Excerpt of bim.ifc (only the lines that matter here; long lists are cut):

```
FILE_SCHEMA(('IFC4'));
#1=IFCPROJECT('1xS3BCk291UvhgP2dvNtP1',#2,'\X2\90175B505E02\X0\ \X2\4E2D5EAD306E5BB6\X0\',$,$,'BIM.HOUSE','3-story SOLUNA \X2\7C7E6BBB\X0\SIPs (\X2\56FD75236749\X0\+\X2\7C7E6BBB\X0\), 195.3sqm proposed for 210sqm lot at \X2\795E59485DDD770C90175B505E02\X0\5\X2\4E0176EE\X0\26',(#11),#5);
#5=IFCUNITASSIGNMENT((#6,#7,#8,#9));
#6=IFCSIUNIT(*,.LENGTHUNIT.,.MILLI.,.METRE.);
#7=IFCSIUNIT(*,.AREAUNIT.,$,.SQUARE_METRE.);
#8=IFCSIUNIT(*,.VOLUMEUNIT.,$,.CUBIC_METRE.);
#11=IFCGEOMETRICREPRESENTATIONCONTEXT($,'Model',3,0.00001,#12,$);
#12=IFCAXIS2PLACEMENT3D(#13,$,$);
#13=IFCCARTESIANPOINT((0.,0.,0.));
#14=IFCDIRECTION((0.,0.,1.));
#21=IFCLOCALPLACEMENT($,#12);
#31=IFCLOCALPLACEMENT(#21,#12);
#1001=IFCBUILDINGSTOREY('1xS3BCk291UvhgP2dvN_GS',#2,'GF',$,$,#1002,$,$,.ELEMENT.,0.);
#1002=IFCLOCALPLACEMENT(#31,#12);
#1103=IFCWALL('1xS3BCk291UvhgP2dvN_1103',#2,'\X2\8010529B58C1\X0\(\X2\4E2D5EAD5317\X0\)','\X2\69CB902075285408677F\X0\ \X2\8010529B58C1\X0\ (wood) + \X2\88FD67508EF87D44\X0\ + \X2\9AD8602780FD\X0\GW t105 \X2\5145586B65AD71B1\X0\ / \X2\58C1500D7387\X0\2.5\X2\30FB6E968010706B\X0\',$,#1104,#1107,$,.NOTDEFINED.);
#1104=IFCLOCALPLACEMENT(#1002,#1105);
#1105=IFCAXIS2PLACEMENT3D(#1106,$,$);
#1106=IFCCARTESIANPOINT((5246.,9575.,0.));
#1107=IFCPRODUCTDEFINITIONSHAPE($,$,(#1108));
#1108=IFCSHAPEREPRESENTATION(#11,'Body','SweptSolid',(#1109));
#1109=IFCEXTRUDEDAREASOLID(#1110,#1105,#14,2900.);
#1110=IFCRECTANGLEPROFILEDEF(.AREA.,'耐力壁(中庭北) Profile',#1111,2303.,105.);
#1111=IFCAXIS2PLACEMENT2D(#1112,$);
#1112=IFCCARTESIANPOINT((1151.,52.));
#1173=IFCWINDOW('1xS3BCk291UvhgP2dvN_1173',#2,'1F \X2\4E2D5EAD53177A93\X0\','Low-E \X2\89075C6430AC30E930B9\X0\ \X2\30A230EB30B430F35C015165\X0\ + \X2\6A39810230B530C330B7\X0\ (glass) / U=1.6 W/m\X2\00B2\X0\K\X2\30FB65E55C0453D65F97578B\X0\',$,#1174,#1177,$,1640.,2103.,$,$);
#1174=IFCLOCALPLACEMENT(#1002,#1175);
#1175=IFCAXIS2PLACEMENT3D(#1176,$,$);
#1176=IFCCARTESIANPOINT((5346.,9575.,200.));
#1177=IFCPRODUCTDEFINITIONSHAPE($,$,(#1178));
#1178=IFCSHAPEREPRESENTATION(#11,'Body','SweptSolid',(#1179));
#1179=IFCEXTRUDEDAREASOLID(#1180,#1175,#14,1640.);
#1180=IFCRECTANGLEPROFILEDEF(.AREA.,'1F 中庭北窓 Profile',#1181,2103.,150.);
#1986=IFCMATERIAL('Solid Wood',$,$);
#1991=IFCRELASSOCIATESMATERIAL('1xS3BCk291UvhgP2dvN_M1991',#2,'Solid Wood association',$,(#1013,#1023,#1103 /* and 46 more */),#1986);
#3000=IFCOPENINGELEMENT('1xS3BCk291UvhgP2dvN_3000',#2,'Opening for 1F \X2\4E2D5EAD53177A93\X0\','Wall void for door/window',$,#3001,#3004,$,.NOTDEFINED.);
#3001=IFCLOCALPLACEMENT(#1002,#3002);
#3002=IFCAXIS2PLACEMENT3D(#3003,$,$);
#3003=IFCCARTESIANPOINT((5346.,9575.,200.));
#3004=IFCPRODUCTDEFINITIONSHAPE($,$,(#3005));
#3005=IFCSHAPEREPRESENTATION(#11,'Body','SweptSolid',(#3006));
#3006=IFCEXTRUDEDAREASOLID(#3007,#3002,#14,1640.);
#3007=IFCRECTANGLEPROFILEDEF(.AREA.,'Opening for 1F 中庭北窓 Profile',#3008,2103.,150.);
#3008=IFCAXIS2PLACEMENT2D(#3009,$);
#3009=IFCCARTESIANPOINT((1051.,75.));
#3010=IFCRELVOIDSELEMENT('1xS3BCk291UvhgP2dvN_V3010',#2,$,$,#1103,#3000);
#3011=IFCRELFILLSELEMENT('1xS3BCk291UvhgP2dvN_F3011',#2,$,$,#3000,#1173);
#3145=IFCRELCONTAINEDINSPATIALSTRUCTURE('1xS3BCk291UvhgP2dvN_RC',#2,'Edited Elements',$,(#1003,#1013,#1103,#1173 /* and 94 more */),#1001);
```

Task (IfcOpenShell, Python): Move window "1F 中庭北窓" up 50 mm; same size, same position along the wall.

```python
import numpy as np
import ifcopenshell
import ifcopenshell.api.geometry
import ifcopenshell.util.placement
import ifcopenshell.util.unit

model = ifcopenshell.open("bim.ifc")
unit_scale = ifcopenshell.util.unit.calculate_unit_scale(model)

window = model.by_guid("1xS3BCk291UvhgP2dvN_1173")
opening = window.FillsVoids[0].RelatingOpeningElement
dz = 50.0

shift = np.array([0.0, 0.0, dz])
# The window is not placed relative to its opening, so move both.
for product in (opening, window):
    matrix = ifcopenshell.util.placement.get_local_placement(product.ObjectPlacement)
    matrix[:3, 3] += shift
    ifcopenshell.api.geometry.edit_object_placement(model, product=product, matrix=matrix, is_si=False)

print(f"moved by {dz * unit_scale:+.3f} m")

model.write("bim_updated.ifc")
```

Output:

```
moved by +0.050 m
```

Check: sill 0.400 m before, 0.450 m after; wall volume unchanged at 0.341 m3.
